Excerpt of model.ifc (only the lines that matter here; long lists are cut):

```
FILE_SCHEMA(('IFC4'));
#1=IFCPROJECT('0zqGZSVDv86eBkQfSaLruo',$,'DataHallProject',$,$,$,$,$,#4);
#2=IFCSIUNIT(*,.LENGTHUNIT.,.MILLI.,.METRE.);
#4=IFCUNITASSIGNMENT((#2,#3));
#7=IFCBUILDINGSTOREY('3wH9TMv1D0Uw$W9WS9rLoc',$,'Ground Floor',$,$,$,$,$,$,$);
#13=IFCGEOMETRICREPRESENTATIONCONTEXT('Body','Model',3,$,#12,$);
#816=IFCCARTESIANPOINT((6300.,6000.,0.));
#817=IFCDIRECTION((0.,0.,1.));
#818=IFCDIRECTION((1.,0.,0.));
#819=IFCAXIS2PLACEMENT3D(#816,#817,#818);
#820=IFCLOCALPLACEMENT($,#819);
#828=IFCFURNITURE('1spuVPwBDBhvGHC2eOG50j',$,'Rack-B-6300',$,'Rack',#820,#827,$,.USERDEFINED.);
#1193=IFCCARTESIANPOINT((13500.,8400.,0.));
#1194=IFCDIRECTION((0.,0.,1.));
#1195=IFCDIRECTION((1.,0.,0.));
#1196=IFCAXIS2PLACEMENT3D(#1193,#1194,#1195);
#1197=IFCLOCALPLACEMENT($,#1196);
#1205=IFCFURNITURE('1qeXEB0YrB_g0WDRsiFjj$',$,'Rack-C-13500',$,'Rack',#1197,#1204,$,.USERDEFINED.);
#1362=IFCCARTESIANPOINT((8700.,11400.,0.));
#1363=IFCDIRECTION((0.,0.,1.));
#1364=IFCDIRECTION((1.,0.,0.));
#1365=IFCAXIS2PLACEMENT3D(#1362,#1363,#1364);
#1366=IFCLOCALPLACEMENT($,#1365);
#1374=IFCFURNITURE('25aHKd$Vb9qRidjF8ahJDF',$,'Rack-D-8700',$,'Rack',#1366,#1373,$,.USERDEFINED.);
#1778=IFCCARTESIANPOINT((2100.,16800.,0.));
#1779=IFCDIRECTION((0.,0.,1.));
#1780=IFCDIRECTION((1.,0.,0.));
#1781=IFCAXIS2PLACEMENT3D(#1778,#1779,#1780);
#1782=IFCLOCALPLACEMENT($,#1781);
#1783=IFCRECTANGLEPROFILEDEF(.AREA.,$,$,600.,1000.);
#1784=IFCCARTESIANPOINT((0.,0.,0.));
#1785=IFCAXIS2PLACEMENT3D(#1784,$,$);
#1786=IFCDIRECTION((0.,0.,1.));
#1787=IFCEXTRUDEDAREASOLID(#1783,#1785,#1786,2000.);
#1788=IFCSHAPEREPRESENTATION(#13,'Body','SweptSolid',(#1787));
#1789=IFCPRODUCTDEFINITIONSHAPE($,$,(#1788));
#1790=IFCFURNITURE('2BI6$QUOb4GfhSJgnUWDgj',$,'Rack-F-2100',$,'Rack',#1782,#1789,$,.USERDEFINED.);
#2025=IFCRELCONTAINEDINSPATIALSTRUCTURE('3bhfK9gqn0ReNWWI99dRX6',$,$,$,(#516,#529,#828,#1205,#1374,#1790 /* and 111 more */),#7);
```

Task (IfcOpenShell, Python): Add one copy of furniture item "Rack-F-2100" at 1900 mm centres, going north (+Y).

```python
import numpy as np
import ifcopenshell
import ifcopenshell.api.geometry
import ifcopenshell.api.root
import ifcopenshell.util.element
import ifcopenshell.util.placement
import ifcopenshell.util.unit

model = ifcopenshell.open("model.ifc")
unit_scale = ifcopenshell.util.unit.calculate_unit_scale(model)

source = model.by_guid("2BI6$QUOb4GfhSJgnUWDgj")
base = ifcopenshell.util.placement.get_local_placement(source.ObjectPlacement)
step = np.array([0.0, 1.0, 0.0]) * 1.9 / unit_scale

for i in range(1, 2):
    copy = ifcopenshell.api.root.copy_class(model, product=source)
    copy.Representation = ifcopenshell.util.element.copy_deep(
        model, source.Representation, exclude=["IfcGeometricRepresentationContext", "IfcRepresentationMap"]
    )
    matrix = base.copy()
    matrix[:3, 3] += i * step
    print("added at", matrix[:3, 3].round(3) + 0.0)
    ifcopenshell.api.geometry.edit_object_placement(model, product=copy, matrix=matrix, is_si=False)

model.write("model_v2.ifc")
```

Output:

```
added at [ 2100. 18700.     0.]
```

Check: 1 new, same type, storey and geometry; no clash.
